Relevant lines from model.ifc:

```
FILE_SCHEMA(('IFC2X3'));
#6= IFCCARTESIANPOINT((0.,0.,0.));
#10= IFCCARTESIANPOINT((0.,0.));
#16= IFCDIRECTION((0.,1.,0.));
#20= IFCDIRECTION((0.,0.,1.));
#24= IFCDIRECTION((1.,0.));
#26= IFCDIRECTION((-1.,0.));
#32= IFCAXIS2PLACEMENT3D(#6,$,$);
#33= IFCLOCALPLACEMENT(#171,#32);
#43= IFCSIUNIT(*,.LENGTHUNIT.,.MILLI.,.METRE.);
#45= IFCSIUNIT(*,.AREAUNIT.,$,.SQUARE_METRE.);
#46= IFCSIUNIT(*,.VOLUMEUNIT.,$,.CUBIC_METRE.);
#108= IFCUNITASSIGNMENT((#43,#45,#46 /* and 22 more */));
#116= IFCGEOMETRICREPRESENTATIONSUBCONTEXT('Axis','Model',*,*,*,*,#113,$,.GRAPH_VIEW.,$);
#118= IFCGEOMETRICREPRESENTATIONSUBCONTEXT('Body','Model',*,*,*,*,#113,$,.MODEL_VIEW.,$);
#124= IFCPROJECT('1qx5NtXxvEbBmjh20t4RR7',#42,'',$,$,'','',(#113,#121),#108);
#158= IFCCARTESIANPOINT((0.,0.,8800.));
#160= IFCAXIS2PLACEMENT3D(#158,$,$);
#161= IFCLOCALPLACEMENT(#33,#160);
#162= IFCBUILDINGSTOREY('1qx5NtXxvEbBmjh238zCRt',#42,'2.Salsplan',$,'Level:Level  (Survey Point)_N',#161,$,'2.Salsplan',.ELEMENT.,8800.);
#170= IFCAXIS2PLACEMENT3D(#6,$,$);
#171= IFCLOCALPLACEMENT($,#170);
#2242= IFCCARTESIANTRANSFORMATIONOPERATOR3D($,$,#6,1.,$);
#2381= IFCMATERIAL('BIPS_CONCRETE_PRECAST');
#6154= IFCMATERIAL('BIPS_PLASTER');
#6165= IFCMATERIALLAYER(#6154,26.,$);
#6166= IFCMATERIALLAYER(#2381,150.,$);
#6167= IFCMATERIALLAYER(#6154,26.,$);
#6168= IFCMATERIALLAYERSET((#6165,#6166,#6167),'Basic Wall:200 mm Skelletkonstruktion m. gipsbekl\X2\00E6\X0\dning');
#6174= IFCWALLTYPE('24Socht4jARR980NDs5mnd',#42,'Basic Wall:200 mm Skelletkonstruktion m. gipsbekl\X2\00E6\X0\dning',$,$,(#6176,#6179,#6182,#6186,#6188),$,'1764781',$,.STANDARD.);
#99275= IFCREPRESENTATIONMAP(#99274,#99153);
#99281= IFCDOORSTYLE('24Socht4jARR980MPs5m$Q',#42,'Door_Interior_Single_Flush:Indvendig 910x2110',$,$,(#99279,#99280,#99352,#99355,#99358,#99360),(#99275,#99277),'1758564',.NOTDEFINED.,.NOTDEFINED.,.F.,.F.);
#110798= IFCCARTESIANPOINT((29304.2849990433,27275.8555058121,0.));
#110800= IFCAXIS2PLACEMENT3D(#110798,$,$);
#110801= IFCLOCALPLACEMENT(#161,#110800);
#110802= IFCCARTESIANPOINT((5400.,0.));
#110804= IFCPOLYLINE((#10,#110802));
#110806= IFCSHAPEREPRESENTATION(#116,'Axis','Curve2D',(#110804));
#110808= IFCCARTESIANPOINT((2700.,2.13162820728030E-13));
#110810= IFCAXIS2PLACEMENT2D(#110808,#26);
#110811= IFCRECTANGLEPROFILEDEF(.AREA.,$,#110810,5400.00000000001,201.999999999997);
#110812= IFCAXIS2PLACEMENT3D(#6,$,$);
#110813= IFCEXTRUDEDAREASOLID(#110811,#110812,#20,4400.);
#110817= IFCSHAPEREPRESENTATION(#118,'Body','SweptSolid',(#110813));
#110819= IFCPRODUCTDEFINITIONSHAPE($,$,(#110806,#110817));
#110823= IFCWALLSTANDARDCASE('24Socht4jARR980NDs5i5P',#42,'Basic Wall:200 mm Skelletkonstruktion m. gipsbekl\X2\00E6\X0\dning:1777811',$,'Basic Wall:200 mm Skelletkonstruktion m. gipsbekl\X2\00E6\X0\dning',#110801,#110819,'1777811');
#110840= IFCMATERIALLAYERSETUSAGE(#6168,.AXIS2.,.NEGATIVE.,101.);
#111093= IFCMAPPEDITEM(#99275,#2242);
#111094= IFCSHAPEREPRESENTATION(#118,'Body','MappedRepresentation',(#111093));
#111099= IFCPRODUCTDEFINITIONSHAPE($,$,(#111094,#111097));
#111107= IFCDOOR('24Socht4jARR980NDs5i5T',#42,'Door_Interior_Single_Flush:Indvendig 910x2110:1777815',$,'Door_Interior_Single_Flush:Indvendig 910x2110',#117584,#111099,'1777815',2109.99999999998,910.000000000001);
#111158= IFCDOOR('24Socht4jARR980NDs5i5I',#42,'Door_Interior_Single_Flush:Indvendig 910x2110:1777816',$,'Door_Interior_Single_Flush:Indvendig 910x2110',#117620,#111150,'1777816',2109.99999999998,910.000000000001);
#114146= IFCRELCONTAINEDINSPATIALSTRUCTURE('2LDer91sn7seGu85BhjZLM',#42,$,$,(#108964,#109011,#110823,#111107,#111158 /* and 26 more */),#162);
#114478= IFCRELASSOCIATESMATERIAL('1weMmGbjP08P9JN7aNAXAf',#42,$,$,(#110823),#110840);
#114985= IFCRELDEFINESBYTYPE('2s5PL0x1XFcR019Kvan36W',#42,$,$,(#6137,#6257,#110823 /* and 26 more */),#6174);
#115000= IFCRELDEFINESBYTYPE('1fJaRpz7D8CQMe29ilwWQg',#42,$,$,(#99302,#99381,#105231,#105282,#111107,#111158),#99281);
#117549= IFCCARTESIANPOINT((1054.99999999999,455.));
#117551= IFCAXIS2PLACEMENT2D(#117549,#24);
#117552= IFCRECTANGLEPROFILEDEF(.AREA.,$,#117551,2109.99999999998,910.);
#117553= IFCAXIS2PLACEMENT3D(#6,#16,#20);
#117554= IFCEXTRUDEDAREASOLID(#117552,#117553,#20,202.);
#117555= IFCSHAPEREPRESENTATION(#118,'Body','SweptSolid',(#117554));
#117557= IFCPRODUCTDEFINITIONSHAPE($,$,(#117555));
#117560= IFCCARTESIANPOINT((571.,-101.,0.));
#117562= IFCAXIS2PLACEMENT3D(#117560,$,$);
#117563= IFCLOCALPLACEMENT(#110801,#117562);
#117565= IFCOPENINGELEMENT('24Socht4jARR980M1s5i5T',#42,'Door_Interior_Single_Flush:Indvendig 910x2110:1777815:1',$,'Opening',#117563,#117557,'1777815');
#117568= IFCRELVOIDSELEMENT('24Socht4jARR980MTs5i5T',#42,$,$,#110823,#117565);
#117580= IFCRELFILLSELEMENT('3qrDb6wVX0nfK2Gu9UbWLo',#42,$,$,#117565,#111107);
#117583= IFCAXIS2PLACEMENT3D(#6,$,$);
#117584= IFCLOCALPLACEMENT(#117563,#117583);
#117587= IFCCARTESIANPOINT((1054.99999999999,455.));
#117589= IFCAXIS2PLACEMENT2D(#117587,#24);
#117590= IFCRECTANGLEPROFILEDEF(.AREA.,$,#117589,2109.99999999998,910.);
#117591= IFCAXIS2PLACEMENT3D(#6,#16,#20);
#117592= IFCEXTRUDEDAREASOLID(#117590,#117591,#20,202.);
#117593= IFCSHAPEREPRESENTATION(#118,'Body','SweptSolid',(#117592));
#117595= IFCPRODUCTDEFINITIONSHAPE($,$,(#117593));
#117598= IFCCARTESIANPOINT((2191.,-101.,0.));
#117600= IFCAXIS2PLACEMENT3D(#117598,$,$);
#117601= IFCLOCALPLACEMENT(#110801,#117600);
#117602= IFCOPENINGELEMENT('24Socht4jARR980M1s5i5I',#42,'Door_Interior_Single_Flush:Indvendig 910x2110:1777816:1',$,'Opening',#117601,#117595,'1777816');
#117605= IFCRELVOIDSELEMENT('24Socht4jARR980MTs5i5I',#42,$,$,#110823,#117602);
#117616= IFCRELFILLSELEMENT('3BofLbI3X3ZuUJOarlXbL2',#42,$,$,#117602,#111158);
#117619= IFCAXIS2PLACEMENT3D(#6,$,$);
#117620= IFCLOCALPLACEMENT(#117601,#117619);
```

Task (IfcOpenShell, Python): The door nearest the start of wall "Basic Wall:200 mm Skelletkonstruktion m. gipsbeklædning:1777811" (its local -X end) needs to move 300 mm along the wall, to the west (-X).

```python
import ifcopenshell
import ifcopenshell.api.geometry
import ifcopenshell.util.placement

model = ifcopenshell.open("model.ifc")

door = model.by_guid("24Socht4jARR980NDs5i5T")
opening = door.FillsVoids[0].RelatingOpeningElement
wall = opening.VoidsElements[0].RelatingBuildingElement

wall_matrix = ifcopenshell.util.placement.get_local_placement(wall.ObjectPlacement)
shift = wall_matrix[:3, 0] * -300.0
before = ifcopenshell.util.placement.get_local_placement(door.ObjectPlacement)[:3, 3].copy()

# The door is placed relative to its opening, so it follows when the opening moves.
matrix = ifcopenshell.util.placement.get_local_placement(opening.ObjectPlacement)
matrix[:3, 3] += shift
ifcopenshell.api.geometry.edit_object_placement(
    model, product=opening, matrix=matrix, is_si=False, should_transform_children=True
)

after = ifcopenshell.util.placement.get_local_placement(door.ObjectPlacement)[:3, 3]
print("door moved by", (after - before).round(3) + 0.0)

model.write("model_updated.ifc")
```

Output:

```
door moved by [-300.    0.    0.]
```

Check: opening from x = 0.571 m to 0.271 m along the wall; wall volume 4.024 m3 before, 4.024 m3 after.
